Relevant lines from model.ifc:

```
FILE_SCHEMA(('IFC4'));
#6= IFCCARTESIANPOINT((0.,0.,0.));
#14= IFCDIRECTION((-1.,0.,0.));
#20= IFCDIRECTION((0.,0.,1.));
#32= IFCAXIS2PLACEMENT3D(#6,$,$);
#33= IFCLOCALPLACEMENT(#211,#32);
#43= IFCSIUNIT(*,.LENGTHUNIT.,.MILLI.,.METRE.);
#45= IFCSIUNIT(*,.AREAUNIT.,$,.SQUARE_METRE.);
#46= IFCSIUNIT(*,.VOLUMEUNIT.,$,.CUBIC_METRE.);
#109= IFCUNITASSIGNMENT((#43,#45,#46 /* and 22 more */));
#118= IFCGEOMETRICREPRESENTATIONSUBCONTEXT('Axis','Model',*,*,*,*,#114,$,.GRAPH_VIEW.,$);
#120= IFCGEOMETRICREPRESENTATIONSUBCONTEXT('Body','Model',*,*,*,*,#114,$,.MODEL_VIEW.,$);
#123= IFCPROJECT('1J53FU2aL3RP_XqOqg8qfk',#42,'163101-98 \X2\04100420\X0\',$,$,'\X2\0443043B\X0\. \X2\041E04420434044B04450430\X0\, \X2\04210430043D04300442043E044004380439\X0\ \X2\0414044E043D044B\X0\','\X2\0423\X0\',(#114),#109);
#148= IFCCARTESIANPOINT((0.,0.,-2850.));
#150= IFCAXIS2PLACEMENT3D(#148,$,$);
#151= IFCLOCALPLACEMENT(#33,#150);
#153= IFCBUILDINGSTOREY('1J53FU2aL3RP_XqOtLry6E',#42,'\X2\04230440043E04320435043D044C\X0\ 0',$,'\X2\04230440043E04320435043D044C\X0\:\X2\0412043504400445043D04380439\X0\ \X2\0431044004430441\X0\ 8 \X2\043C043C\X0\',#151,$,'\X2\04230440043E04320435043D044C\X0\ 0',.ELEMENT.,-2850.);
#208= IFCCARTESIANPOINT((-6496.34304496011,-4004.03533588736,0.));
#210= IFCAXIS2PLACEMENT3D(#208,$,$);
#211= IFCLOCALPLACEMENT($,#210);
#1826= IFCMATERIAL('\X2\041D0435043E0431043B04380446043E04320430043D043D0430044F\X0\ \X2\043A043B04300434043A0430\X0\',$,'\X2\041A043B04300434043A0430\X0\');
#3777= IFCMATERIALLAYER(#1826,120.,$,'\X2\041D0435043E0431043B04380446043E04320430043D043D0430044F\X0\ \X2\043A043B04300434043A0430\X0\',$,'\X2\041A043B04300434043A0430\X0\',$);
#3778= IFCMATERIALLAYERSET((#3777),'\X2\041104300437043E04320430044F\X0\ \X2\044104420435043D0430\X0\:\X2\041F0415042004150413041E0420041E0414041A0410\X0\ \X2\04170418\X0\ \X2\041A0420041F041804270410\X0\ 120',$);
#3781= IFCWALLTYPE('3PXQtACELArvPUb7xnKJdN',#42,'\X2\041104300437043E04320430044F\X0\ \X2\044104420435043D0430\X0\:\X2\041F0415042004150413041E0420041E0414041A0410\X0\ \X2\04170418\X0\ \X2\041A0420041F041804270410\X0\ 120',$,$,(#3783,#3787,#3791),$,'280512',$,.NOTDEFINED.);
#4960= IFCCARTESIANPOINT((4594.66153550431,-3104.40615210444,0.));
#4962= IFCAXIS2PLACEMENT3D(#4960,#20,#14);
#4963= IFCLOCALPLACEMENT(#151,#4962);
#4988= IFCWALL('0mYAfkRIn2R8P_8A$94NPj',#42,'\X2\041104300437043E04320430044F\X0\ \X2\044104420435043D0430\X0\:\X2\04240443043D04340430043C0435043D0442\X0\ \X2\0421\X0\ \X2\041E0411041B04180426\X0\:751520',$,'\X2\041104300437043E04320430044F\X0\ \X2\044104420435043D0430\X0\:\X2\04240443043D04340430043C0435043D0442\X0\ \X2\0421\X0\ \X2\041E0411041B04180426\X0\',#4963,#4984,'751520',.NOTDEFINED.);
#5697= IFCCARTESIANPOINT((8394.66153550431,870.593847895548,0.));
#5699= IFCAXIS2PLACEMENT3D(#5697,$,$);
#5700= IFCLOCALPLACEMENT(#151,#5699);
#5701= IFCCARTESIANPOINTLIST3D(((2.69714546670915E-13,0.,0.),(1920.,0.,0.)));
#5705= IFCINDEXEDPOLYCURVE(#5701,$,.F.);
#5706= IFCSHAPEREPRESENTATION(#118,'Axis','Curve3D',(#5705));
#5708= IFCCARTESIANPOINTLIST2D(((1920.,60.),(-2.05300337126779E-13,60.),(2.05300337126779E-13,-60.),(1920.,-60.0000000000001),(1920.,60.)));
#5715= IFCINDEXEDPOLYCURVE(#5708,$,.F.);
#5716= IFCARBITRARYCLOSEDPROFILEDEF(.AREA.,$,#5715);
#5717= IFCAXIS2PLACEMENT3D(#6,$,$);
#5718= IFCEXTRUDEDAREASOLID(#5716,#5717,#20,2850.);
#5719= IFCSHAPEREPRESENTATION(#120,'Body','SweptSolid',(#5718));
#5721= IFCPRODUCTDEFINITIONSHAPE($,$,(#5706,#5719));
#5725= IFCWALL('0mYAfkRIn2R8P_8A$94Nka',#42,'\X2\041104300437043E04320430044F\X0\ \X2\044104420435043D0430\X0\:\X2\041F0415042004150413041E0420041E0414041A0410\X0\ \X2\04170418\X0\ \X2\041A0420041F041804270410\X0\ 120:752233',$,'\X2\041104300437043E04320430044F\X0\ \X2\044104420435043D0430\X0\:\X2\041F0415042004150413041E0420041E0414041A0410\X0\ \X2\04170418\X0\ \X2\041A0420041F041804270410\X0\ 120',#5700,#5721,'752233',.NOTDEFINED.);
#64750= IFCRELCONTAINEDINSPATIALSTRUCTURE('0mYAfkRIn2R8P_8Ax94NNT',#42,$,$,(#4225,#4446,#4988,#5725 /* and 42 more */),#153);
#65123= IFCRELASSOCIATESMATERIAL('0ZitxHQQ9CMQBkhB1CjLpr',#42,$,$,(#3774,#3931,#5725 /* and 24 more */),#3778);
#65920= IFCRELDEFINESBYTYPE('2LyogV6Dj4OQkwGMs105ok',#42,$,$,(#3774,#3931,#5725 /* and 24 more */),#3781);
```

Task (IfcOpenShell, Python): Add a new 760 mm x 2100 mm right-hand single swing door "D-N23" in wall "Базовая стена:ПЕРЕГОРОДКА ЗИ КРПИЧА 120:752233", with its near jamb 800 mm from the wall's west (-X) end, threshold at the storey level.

```python
import numpy as np
import ifcopenshell
import ifcopenshell.api.feature
import ifcopenshell.api.geometry
import ifcopenshell.api.root
import ifcopenshell.api.spatial
import ifcopenshell.geom
import ifcopenshell.util.element
import ifcopenshell.util.placement
import ifcopenshell.util.representation
import ifcopenshell.util.shape
import ifcopenshell.util.unit

model = ifcopenshell.open("model.ifc")
unit_scale = ifcopenshell.util.unit.calculate_unit_scale(model)
settings = ifcopenshell.geom.settings()


def volume(element):
    """Net volume in cubic metres, openings subtracted."""
    shape = ifcopenshell.geom.create_shape(settings, element)
    return ifcopenshell.util.shape.get_volume(shape.geometry)


wall = model.by_guid("0mYAfkRIn2R8P_8A$94Nka")
storey = ifcopenshell.util.element.get_container(wall, ifc_class="IfcBuildingStorey")
context = ifcopenshell.util.representation.get_context(model, "Model", "Body", "MODEL_VIEW")
before = volume(wall)

width, height, from_end, sill = 0.76, 2.1, 0.8, 0.0  # metres

# The wall runs along its own X axis, and the end named is its -X end.
wall_shape = ifcopenshell.geom.create_shape(settings, wall)
x, y, z = ifcopenshell.util.shape.get_vertices(wall_shape.geometry).T
start = x.min() + from_end
face, thickness = float(y.min()), float(y.max() - y.min())
wall_matrix = ifcopenshell.util.placement.get_local_placement(wall.ObjectPlacement)
level = ifcopenshell.util.placement.get_local_placement(storey.ObjectPlacement)[2, 3]


def in_wall(x, y):
    """Placement at x, y metres in the wall's axes, at sill height."""
    matrix = wall_matrix.copy()
    matrix[:, 3] = wall_matrix @ np.array([x / unit_scale, y / unit_scale, 0.0, 1.0])
    matrix[2, 3] = level + sill / unit_scale
    return matrix


# Opening: a box that overshoots both wall faces by 50 mm.
opening = ifcopenshell.api.root.create_entity(model, ifc_class="IfcOpeningElement", predefined_type="OPENING")
box = ifcopenshell.api.geometry.add_wall_representation(
    model, context=context, length=width, height=height, thickness=thickness + 0.1
)
ifcopenshell.api.geometry.assign_representation(model, product=opening, representation=box)
ifcopenshell.api.geometry.edit_object_placement(model, product=opening, matrix=in_wall(start, face - 0.05), is_si=False)
ifcopenshell.api.feature.add_feature(model, feature=opening, element=wall)

door = ifcopenshell.api.root.create_entity(model, ifc_class="IfcDoor", name="D-N23", predefined_type="DOOR")
door.OverallWidth, door.OverallHeight = width / unit_scale, height / unit_scale
door.OperationType = "SINGLE_SWING_RIGHT"
body = ifcopenshell.api.geometry.add_door_representation(
    model,
    context=context,
    overall_width=door.OverallWidth,
    overall_height=door.OverallHeight,
    operation_type="SINGLE_SWING_RIGHT",
    lining_properties={"LiningDepth": thickness / unit_scale, "ThresholdDepth": thickness / unit_scale},
)
ifcopenshell.api.geometry.assign_representation(model, product=door, representation=body)
ifcopenshell.api.spatial.assign_container(model, products=[door], relating_structure=storey)
ifcopenshell.api.feature.add_filling(model, opening=opening, element=door)

# The lining spans the wall, so the door starts at the wall face.
ifcopenshell.api.geometry.edit_object_placement(model, product=door, matrix=in_wall(start, face), is_si=False)

after = volume(wall)

print(f"wall volume {before:.3f} -> {after:.3f} m3")

model.write("model_rev.ifc")
```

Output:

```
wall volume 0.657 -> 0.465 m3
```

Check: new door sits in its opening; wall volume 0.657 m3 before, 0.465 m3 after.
